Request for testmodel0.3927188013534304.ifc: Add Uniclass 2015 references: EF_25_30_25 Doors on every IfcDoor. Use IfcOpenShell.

First a look at what the model holds.

```python
import ifcopenshell

model = ifcopenshell.open("testmodel0.3927188013534304.ifc")
print(model.schema)
print("classifications:", [c.Name for c in model.by_type("IfcClassification")])
for ifc_class in ("IfcDoor", "IfcRoof", "IfcStair", "IfcWall", "IfcWindow"):
    print(ifc_class, len(model.by_type(ifc_class)))
```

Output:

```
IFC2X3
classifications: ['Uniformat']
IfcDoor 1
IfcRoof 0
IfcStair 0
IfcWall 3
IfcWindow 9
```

```python
import ifcopenshell
import ifcopenshell.api.classification

model = ifcopenshell.open("testmodel0.3927188013534304.ifc")

# IFC2X3 requires Source and Edition and has no link from the project to the system.
system = model.create_entity("IfcClassification", Source="NBS", Edition="2015", Name="Uniclass 2015")

codes = {
    "IfcDoor": ("EF_25_30_25", "Doors"),
}
for ifc_class, (code, name) in codes.items():
    products = model.by_type(ifc_class)
    ifcopenshell.api.classification.add_reference(
        model, products=products, classification=system, identification=code, name=name
    )
    print(code, len(products))

model.write("testmodel0.3927188013534304_rev.ifc")
```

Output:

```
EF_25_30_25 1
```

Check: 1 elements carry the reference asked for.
